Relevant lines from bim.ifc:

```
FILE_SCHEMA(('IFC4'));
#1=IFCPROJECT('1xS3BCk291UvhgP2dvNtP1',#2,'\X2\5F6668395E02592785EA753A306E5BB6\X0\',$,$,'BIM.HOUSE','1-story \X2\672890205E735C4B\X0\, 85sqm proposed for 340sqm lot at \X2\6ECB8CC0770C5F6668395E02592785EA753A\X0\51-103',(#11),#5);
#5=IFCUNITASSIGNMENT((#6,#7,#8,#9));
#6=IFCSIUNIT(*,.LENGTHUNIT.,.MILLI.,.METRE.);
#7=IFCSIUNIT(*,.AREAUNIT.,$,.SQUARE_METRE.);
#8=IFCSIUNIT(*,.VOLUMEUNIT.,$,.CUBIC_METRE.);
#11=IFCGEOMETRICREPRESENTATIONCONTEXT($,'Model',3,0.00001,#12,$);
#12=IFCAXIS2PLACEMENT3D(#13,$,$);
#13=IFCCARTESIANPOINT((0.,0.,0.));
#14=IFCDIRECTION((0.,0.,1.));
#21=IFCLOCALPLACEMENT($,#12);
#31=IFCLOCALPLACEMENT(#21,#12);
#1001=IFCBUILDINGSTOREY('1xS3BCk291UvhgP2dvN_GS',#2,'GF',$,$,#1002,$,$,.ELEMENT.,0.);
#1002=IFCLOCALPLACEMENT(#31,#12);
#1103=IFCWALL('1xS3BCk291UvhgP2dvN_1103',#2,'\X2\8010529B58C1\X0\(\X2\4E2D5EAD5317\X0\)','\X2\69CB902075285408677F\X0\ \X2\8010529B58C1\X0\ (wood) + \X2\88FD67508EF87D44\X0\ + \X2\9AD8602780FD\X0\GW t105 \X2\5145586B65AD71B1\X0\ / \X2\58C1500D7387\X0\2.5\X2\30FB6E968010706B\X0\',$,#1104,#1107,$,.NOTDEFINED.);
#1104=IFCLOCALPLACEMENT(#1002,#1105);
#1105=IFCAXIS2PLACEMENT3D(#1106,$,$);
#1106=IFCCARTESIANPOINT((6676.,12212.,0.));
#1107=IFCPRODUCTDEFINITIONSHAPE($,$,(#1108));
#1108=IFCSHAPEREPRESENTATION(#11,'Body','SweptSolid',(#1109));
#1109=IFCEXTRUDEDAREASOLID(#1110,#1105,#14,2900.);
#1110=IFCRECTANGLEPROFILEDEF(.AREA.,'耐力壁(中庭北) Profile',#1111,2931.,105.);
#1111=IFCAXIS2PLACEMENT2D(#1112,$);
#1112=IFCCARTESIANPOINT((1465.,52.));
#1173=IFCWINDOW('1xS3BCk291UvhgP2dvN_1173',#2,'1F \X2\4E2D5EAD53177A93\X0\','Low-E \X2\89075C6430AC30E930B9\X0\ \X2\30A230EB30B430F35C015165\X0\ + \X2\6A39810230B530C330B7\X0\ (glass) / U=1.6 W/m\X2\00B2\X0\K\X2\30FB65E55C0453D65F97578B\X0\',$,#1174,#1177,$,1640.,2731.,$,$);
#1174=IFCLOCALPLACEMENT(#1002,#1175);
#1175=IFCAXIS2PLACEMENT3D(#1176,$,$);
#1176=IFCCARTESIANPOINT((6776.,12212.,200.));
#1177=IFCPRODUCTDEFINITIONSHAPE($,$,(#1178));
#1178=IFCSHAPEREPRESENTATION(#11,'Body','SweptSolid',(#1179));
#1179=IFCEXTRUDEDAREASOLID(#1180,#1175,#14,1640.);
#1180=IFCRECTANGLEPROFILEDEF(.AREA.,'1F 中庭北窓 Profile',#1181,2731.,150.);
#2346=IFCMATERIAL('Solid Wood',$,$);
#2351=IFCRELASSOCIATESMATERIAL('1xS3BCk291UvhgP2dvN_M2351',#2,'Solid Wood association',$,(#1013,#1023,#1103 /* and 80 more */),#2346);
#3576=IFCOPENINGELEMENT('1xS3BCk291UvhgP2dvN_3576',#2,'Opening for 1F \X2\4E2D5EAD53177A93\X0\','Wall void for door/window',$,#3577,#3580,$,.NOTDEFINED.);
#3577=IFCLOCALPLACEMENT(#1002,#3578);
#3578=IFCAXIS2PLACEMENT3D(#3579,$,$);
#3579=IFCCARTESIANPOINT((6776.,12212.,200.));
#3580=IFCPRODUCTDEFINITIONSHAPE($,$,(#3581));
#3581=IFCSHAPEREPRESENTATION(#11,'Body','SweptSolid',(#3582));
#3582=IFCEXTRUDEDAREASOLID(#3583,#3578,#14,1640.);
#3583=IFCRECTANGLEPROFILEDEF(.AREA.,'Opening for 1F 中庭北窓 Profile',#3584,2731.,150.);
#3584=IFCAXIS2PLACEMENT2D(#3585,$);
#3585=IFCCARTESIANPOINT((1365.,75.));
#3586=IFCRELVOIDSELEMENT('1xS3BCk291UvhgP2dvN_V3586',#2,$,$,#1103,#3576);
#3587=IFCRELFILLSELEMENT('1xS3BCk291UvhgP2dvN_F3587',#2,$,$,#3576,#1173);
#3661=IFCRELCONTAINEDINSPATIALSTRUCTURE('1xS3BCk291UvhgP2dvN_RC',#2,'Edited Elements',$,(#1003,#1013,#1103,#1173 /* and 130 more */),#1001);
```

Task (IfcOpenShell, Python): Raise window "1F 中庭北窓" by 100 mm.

```python
import numpy as np
import ifcopenshell
import ifcopenshell.api.geometry
import ifcopenshell.util.placement
import ifcopenshell.util.unit

model = ifcopenshell.open("bim.ifc")
unit_scale = ifcopenshell.util.unit.calculate_unit_scale(model)

window = model.by_id(1173)
opening = window.FillsVoids[0].RelatingOpeningElement
dz = 100.0

shift = np.array([0.0, 0.0, dz])
# The window is not placed relative to its opening, so move both.
for product in (opening, window):
    matrix = ifcopenshell.util.placement.get_local_placement(product.ObjectPlacement)
    matrix[:3, 3] += shift
    ifcopenshell.api.geometry.edit_object_placement(model, product=product, matrix=matrix, is_si=False)

print(f"moved by {dz * unit_scale:+.3f} m")

model.write("bim_updated.ifc")
```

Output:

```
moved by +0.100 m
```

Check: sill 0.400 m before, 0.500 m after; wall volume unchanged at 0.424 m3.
